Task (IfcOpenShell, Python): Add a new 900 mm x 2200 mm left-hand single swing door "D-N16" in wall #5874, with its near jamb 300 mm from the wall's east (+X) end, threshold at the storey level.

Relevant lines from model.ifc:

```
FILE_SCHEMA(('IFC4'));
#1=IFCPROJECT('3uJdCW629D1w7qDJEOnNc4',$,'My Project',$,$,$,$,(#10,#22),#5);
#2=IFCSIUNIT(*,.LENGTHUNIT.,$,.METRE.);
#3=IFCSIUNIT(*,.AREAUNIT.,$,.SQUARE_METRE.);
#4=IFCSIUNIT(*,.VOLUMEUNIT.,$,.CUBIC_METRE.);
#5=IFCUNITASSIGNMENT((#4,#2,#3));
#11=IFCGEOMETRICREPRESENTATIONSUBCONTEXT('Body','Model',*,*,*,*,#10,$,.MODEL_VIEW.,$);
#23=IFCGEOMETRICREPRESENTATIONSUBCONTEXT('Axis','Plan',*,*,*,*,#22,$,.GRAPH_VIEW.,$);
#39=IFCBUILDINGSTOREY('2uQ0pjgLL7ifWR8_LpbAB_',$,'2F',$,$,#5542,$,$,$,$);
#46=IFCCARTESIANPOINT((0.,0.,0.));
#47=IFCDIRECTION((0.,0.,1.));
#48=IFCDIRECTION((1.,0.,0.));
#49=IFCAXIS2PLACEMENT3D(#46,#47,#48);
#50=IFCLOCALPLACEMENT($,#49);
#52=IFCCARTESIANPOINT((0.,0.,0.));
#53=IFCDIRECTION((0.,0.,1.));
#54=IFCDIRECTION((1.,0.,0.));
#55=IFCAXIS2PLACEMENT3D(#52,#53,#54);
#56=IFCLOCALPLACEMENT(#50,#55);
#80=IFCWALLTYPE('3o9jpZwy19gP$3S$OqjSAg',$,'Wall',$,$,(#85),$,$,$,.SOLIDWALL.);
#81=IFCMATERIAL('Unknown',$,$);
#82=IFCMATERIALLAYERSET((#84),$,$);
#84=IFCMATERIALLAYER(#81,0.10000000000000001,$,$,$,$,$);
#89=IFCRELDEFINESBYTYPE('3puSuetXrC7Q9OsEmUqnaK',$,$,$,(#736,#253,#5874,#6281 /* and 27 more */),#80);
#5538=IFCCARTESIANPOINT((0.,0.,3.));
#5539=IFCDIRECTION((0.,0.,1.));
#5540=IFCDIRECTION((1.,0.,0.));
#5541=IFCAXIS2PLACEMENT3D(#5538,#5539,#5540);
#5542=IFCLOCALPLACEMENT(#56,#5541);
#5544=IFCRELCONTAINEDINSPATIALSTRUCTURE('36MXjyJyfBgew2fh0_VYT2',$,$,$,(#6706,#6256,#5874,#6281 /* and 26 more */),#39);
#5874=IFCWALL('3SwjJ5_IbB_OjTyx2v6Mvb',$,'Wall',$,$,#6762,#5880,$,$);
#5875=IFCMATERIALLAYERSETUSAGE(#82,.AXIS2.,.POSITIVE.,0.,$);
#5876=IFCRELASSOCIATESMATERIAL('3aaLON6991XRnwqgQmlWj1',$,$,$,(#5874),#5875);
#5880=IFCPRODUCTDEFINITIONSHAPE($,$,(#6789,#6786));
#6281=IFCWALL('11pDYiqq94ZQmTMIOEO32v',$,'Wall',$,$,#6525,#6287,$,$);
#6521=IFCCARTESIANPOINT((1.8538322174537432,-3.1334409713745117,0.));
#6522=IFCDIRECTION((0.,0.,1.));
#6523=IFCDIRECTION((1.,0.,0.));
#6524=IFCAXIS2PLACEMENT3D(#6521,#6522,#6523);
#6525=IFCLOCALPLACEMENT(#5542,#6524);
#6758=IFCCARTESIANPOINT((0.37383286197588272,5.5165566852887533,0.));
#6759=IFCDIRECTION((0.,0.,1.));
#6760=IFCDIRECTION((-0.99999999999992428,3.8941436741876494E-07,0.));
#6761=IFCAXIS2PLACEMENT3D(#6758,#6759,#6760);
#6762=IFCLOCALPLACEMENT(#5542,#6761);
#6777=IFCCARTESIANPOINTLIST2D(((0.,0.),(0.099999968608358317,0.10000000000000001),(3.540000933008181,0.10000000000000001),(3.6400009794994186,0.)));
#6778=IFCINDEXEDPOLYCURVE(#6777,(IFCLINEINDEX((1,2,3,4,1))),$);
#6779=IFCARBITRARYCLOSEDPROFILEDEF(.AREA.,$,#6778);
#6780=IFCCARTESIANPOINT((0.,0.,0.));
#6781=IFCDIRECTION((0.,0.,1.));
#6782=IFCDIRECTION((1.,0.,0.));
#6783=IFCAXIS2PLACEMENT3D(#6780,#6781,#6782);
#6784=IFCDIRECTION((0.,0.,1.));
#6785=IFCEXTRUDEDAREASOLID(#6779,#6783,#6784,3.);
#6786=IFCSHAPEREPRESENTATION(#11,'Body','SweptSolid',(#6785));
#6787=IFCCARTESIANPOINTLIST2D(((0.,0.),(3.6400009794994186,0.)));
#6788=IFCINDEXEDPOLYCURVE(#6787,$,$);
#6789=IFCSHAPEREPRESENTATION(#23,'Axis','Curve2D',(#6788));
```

```python
import numpy as np
import ifcopenshell
import ifcopenshell.api.feature
import ifcopenshell.api.geometry
import ifcopenshell.api.root
import ifcopenshell.api.spatial
import ifcopenshell.geom
import ifcopenshell.util.element
import ifcopenshell.util.placement
import ifcopenshell.util.representation
import ifcopenshell.util.shape
import ifcopenshell.util.unit

model = ifcopenshell.open("model.ifc")
unit_scale = ifcopenshell.util.unit.calculate_unit_scale(model)
settings = ifcopenshell.geom.settings()


def volume(element):
    """Net volume in cubic metres, openings subtracted."""
    shape = ifcopenshell.geom.create_shape(settings, element)
    return ifcopenshell.util.shape.get_volume(shape.geometry)


wall = model.by_guid("3SwjJ5_IbB_OjTyx2v6Mvb")
storey = ifcopenshell.util.element.get_container(wall, ifc_class="IfcBuildingStorey")
context = ifcopenshell.util.representation.get_context(model, "Model", "Body", "MODEL_VIEW")
before = volume(wall)

width, height, from_end, sill = 0.9, 2.2, 0.3, 0.0  # metres

# The wall runs along its own X axis, and the end named is its -X end.
wall_shape = ifcopenshell.geom.create_shape(settings, wall)
x, y, z = ifcopenshell.util.shape.get_vertices(wall_shape.geometry).T
start = x.min() + from_end
face, thickness = float(y.min()), float(y.max() - y.min())
wall_matrix = ifcopenshell.util.placement.get_local_placement(wall.ObjectPlacement)
level = ifcopenshell.util.placement.get_local_placement(storey.ObjectPlacement)[2, 3]


def in_wall(x, y):
    """Placement at x, y metres in the wall's axes, at sill height."""
    matrix = wall_matrix.copy()
    matrix[:, 3] = wall_matrix @ np.array([x / unit_scale, y / unit_scale, 0.0, 1.0])
    matrix[2, 3] = level + sill / unit_scale
    return matrix


# Opening: a box that overshoots both wall faces by 50 mm.
opening = ifcopenshell.api.root.create_entity(model, ifc_class="IfcOpeningElement", predefined_type="OPENING")
box = ifcopenshell.api.geometry.add_wall_representation(
    model, context=context, length=width, height=height, thickness=thickness + 0.1
)
ifcopenshell.api.geometry.assign_representation(model, product=opening, representation=box)
ifcopenshell.api.geometry.edit_object_placement(model, product=opening, matrix=in_wall(start, face - 0.05), is_si=False)
ifcopenshell.api.feature.add_feature(model, feature=opening, element=wall)

door = ifcopenshell.api.root.create_entity(model, ifc_class="IfcDoor", name="D-N16", predefined_type="DOOR")
door.OverallWidth, door.OverallHeight = width / unit_scale, height / unit_scale
door.OperationType = "SINGLE_SWING_LEFT"
body = ifcopenshell.api.geometry.add_door_representation(
    model,
    context=context,
    overall_width=door.OverallWidth,
    overall_height=door.OverallHeight,
    operation_type="SINGLE_SWING_LEFT",
    lining_properties={"LiningDepth": thickness / unit_scale, "ThresholdDepth": thickness / unit_scale},
)
ifcopenshell.api.geometry.assign_representation(model, product=door, representation=body)
ifcopenshell.api.spatial.assign_container(model, products=[door], relating_structure=storey)
ifcopenshell.api.feature.add_filling(model, opening=opening, element=door)

# The lining spans the wall, so the door starts at the wall face.
ifcopenshell.api.geometry.edit_object_placement(model, product=door, matrix=in_wall(start, face), is_si=False)

after = volume(wall)

print(f"wall volume {before:.3f} -> {after:.3f} m3")

model.write("model_edited.ifc")
```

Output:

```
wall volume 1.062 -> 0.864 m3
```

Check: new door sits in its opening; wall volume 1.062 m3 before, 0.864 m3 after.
